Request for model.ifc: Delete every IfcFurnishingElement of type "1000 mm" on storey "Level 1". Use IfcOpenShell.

First a look at what the model holds.

```python
import ifcopenshell
import ifcopenshell.util.element

model = ifcopenshell.open("model.ifc")
print(model.schema)
storey = next(s for s in model.by_type("IfcBuildingStorey") if s.Name == "Level 1")
furniture = [e for e in ifcopenshell.util.element.get_decomposition(storey) if e.is_a("IfcFurnishingElement")]
seen = {}
for e in furniture:
    element_type = ifcopenshell.util.element.get_type(e)
    name = element_type.Name if element_type not in (None, e) else None
    seen[name] = seen.get(name, 0) + 1
for name, count in sorted(seen.items(), key=str):
    print(count, "x", name)
```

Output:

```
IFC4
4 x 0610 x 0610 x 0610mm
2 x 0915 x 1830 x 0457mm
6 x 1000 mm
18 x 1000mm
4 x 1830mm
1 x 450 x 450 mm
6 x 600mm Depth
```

```python
import ifcopenshell
import ifcopenshell.api.root
import ifcopenshell.util.element

model = ifcopenshell.open("model.ifc")

storey = next(s for s in model.by_type("IfcBuildingStorey") if s.Name == "Level 1")
furniture = [e for e in ifcopenshell.util.element.get_decomposition(storey) if e.is_a("IfcFurnishingElement")]
targets = [e for e in furniture if (t := ifcopenshell.util.element.get_type(e)) not in (None, e) and t.Name == "1000 mm"]

for e in targets:
    ifcopenshell.api.root.remove_product(model, product=e)
print(len(targets), "removed")

model.write("model_rev.ifc")
```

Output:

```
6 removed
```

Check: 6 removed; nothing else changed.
